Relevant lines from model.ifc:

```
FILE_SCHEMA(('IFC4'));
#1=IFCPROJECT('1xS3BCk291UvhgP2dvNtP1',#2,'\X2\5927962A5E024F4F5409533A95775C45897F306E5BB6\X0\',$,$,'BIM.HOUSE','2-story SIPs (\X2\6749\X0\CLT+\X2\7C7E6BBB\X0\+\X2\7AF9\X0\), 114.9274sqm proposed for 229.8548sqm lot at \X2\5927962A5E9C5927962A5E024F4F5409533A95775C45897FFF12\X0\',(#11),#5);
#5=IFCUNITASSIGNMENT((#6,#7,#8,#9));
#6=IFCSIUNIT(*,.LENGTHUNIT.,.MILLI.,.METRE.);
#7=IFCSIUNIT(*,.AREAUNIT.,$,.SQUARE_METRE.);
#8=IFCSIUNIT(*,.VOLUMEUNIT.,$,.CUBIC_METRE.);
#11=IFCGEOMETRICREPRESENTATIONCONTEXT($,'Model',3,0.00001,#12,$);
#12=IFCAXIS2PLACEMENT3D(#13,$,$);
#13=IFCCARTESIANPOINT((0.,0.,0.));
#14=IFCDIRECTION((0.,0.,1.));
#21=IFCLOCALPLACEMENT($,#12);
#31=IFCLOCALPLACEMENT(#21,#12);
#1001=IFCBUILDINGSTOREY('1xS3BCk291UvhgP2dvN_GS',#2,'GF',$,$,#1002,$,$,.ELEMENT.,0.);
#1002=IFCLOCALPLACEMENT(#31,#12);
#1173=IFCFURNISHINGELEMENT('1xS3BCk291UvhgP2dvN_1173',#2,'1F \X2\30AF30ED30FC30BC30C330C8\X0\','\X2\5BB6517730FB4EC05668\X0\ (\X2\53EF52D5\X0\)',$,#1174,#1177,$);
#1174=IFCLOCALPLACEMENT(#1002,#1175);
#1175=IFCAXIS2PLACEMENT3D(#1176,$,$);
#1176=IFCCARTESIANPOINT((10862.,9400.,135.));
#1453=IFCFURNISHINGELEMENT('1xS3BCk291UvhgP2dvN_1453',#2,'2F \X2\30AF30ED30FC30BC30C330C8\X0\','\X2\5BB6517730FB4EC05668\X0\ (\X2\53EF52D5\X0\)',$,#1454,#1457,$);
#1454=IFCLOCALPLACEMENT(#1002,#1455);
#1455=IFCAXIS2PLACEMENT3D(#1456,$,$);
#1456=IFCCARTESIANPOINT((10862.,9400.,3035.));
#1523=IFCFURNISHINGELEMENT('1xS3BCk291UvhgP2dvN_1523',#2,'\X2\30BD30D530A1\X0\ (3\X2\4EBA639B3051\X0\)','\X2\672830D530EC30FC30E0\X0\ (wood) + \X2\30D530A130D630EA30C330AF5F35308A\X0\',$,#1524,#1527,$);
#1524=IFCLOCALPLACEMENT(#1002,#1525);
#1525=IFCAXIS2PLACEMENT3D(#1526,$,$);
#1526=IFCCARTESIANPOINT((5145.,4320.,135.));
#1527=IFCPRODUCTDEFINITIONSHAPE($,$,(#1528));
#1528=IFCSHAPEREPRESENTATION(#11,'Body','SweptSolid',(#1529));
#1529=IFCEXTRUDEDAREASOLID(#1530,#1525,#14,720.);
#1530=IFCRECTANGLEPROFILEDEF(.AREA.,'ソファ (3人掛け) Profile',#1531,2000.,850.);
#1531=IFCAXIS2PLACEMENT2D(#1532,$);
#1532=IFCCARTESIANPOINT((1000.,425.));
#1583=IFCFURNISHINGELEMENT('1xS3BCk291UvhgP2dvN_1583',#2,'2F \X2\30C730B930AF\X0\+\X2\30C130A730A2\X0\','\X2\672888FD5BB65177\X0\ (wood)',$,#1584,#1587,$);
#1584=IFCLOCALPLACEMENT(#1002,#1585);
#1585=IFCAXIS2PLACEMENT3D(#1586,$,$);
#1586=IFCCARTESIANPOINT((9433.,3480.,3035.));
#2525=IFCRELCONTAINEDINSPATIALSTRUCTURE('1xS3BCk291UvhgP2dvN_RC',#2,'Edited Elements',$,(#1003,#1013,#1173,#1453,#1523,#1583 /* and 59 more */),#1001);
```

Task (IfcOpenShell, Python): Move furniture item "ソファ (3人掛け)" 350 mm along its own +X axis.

```python
import ifcopenshell
import ifcopenshell.api.geometry
import ifcopenshell.util.placement
import ifcopenshell.util.unit

model = ifcopenshell.open("model.ifc")
unit_scale = ifcopenshell.util.unit.calculate_unit_scale(model)

item = model.by_id(1523)
matrix = ifcopenshell.util.placement.get_local_placement(item.ObjectPlacement)
matrix[:3, 3] += matrix[:3, 0] * 0.35 / unit_scale
ifcopenshell.api.geometry.edit_object_placement(model, product=item, matrix=matrix, is_si=False)

print(ifcopenshell.util.placement.get_local_placement(item.ObjectPlacement).round(3) + 0.0)

model.write("model_updated.ifc")
```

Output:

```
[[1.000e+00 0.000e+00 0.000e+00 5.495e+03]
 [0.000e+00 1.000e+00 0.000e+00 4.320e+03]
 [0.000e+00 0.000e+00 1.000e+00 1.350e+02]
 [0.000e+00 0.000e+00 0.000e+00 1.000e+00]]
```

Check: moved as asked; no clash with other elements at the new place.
